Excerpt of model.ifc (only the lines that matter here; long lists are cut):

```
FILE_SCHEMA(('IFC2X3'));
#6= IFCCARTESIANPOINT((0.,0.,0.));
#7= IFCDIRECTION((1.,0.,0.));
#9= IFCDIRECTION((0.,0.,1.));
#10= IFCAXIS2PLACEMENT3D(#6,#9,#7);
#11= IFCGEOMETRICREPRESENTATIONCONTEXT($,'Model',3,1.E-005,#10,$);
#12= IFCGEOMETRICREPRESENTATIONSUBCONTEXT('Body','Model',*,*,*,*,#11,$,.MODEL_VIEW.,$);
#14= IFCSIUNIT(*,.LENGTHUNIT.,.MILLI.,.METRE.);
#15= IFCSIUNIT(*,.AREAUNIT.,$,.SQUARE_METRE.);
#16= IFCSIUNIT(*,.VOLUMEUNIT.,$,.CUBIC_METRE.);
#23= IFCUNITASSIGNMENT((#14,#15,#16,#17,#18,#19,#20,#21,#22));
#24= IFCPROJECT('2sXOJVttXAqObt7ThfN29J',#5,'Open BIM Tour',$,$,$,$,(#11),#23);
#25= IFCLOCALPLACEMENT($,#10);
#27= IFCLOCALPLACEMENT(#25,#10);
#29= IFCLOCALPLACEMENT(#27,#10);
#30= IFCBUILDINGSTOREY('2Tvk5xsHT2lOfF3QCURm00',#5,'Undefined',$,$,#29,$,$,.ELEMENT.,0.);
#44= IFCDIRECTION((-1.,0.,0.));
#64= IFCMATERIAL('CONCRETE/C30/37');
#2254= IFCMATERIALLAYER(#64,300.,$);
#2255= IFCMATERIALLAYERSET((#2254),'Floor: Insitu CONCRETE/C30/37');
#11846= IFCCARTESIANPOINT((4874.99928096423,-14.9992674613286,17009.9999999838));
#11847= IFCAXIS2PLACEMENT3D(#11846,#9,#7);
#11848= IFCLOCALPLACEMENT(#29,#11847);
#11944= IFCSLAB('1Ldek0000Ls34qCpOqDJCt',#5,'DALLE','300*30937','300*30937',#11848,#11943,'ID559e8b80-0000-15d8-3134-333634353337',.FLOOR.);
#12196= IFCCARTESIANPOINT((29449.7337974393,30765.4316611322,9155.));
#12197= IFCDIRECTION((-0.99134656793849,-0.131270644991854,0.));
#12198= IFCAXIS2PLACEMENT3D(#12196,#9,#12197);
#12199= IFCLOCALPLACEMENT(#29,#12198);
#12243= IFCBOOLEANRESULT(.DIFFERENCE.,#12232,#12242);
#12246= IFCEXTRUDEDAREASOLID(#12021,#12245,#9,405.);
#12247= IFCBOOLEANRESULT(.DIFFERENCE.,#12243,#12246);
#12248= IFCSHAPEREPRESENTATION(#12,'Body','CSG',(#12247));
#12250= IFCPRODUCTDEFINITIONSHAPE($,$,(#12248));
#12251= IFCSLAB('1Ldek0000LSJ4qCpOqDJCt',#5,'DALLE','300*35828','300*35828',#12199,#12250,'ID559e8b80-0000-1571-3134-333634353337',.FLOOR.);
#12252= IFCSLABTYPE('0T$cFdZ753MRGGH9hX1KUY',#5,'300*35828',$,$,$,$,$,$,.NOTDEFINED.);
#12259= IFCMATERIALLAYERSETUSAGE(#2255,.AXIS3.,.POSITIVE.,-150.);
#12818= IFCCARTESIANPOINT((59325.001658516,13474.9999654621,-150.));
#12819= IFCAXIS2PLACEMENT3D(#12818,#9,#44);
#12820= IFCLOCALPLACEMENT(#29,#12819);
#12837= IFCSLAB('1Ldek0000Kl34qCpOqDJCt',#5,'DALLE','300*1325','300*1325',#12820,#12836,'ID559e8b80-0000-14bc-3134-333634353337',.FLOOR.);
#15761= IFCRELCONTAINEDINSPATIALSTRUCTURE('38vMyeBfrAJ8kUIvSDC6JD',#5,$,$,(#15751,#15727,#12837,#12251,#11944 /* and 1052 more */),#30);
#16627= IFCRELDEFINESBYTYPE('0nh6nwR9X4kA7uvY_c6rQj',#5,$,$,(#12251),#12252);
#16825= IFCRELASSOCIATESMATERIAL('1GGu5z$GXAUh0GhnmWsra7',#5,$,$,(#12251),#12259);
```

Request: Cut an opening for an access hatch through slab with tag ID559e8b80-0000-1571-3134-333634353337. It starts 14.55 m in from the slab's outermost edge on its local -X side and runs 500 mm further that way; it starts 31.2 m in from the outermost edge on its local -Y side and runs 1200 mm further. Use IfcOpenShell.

```python
import numpy as np
import ifcopenshell
import ifcopenshell.api.feature
import ifcopenshell.api.geometry
import ifcopenshell.api.root
import ifcopenshell.geom
import ifcopenshell.util.placement
import ifcopenshell.util.representation
import ifcopenshell.util.shape
import ifcopenshell.util.unit

model = ifcopenshell.open("model.ifc")
unit_scale = ifcopenshell.util.unit.calculate_unit_scale(model)
settings = ifcopenshell.geom.settings()


def volume(element):
    """Net volume in cubic metres, openings subtracted."""
    shape = ifcopenshell.geom.create_shape(settings, element)
    return ifcopenshell.util.shape.get_volume(shape.geometry)


slab = model.by_id(12251)
before = volume(slab)

# Extent in the slab's own axes, in metres. The edges named are its -X and -Y sides.
slab_shape = ifcopenshell.geom.create_shape(settings, slab)
vertices = ifcopenshell.util.shape.get_vertices(slab_shape.geometry)
x_min, y_min, bottom = vertices.min(axis=0)
top = vertices[:, 2].max()

opening = ifcopenshell.api.root.create_entity(model, ifc_class="IfcOpeningElement", name="Access hatch opening")
context = ifcopenshell.util.representation.get_context(model, "Model", "Body", "MODEL_VIEW")
width, depth = 0.5, 1.2
outline = [(0.0, 0.0), (width, 0.0), (width, depth), (0.0, depth), (0.0, 0.0)]
# Overshoot both faces by 50 mm so the cut is clean.
shape = ifcopenshell.api.geometry.add_slab_representation(
    model, context=context, depth=top - bottom + 0.1, polyline=outline
)
ifcopenshell.api.geometry.assign_representation(model, product=opening, representation=shape)

matrix = ifcopenshell.util.placement.get_local_placement(slab.ObjectPlacement)
matrix[:, 3] = matrix @ np.append(np.array([x_min + 14.55, y_min + 31.2, bottom - 0.05]) / unit_scale, 1.0)
ifcopenshell.api.geometry.edit_object_placement(model, product=opening, matrix=matrix, is_si=False)
ifcopenshell.api.feature.add_feature(model, feature=opening, element=slab)

after = volume(slab)

print(f"slab volume {before:.3f} -> {after:.3f} m3")

model.write("model_updated.ifc")
```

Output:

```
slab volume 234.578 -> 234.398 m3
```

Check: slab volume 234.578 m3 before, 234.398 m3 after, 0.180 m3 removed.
